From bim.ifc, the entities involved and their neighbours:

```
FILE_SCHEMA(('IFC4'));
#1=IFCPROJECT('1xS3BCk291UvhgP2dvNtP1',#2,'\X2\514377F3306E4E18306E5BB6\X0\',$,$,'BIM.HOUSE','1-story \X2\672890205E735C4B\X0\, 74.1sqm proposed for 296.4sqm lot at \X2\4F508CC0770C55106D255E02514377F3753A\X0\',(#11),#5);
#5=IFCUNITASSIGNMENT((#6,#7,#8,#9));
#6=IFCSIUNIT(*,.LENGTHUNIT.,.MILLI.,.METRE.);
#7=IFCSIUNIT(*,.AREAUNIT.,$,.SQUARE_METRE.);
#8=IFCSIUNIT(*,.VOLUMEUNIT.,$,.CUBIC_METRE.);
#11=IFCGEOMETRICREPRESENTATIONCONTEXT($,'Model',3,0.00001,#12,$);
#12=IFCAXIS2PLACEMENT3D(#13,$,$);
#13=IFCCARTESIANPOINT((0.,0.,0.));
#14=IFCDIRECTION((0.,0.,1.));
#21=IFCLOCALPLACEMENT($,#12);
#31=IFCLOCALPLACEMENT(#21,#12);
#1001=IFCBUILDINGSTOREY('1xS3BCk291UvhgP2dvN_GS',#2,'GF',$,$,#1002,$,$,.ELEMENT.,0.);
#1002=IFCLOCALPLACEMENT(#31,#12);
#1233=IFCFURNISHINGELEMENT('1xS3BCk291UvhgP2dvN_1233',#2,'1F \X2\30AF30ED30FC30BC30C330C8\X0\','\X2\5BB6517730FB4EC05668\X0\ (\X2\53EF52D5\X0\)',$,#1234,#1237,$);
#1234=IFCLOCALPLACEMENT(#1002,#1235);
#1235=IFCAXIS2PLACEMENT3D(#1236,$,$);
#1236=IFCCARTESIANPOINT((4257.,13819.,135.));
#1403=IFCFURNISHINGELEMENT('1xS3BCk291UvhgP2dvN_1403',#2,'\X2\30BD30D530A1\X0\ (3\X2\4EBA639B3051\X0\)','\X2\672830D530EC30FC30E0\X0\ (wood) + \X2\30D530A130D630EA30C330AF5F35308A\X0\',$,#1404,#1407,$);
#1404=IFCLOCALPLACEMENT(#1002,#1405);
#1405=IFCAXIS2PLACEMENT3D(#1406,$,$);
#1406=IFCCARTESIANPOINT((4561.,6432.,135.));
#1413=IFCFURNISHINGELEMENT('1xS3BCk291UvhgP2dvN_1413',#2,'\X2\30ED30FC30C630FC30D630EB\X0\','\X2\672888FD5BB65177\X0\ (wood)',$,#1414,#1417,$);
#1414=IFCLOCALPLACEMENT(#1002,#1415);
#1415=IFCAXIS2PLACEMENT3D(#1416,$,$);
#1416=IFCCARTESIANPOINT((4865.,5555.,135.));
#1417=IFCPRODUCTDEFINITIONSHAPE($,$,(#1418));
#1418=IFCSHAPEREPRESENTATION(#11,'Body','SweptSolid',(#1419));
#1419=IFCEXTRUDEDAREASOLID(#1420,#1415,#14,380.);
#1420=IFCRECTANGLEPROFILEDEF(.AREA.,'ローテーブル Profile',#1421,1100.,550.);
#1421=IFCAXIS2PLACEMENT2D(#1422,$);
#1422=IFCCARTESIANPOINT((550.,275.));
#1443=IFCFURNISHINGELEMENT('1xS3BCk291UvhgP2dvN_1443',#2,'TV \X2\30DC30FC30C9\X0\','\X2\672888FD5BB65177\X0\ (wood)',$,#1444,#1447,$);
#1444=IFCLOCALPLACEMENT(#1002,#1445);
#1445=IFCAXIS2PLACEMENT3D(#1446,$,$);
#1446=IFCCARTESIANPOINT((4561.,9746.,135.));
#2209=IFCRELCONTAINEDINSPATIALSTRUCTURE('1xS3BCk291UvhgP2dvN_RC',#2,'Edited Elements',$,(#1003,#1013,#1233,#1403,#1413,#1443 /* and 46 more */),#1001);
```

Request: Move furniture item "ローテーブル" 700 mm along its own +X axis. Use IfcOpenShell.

```python
import ifcopenshell
import ifcopenshell.api.geometry
import ifcopenshell.util.placement
import ifcopenshell.util.unit

model = ifcopenshell.open("bim.ifc")
unit_scale = ifcopenshell.util.unit.calculate_unit_scale(model)

item = model.by_guid("1xS3BCk291UvhgP2dvN_1413")
matrix = ifcopenshell.util.placement.get_local_placement(item.ObjectPlacement)
matrix[:3, 3] += matrix[:3, 0] * 0.7 / unit_scale
ifcopenshell.api.geometry.edit_object_placement(model, product=item, matrix=matrix, is_si=False)

print(ifcopenshell.util.placement.get_local_placement(item.ObjectPlacement).round(3) + 0.0)

model.write("bim_v2.ifc")
```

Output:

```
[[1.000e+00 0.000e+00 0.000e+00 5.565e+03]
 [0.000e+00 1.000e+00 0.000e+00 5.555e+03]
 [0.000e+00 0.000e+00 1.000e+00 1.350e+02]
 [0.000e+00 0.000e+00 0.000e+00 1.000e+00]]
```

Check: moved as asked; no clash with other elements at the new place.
